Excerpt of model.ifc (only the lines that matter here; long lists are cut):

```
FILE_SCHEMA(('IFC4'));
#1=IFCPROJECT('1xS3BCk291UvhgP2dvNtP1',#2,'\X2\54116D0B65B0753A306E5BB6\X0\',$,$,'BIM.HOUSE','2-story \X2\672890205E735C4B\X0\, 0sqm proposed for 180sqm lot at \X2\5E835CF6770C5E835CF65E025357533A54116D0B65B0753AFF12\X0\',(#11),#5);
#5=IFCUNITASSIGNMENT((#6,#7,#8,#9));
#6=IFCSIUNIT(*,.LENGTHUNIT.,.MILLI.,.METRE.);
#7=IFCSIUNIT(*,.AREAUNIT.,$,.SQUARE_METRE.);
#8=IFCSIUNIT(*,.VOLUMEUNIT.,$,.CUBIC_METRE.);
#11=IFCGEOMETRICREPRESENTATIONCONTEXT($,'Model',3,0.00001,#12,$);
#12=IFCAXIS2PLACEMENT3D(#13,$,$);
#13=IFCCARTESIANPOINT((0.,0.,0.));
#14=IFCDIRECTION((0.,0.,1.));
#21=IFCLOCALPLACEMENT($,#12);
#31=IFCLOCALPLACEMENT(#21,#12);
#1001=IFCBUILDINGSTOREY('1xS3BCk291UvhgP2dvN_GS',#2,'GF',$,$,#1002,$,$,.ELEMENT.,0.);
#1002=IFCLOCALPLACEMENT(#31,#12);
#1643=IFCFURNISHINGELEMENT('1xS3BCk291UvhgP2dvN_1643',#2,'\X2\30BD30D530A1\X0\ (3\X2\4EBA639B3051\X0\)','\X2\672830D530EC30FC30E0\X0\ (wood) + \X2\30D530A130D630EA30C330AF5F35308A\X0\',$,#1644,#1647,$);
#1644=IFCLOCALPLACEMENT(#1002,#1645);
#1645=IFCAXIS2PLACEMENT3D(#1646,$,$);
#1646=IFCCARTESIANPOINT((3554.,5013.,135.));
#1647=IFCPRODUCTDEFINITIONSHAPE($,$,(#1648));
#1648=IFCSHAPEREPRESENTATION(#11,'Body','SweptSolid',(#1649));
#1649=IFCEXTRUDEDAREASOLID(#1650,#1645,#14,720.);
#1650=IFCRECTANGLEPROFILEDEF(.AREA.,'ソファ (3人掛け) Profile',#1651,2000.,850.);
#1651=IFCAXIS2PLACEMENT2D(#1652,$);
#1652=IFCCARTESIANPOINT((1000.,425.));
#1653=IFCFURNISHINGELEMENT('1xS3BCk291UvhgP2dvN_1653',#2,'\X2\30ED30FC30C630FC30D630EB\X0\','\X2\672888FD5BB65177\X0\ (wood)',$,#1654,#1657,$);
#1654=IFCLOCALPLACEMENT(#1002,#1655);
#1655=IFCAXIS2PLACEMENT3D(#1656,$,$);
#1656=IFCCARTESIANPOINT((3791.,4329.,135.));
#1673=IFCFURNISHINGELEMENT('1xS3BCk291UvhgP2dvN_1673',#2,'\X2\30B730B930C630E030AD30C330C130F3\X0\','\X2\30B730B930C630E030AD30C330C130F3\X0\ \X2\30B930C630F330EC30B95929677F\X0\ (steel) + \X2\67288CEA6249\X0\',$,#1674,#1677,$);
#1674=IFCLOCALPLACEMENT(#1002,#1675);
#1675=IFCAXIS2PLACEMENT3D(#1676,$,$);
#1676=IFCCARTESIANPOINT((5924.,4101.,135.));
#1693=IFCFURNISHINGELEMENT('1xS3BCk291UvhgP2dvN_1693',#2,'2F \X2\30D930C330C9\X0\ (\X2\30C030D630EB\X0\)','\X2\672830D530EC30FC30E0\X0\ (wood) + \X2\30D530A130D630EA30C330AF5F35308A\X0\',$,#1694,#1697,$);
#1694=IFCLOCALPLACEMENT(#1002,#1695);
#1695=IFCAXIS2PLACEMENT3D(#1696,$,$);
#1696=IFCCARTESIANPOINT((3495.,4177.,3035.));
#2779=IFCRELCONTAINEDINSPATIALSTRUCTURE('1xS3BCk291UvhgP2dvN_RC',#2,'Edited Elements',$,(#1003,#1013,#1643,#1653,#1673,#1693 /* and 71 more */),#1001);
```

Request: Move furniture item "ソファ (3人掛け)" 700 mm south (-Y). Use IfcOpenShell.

```python
import ifcopenshell
import ifcopenshell.api.geometry
import ifcopenshell.util.placement

model = ifcopenshell.open("model.ifc")

item = model.by_guid("1xS3BCk291UvhgP2dvN_1643")
matrix = ifcopenshell.util.placement.get_local_placement(item.ObjectPlacement)
matrix[1, 3] -= 700.0
ifcopenshell.api.geometry.edit_object_placement(model, product=item, matrix=matrix, is_si=False)

print(ifcopenshell.util.placement.get_local_placement(item.ObjectPlacement).round(3) + 0.0)

model.write("model_rev.ifc")
```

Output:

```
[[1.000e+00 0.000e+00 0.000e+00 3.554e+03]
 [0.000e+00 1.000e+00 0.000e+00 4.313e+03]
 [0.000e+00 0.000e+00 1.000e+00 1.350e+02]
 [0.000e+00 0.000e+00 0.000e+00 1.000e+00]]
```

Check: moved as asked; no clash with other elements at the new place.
